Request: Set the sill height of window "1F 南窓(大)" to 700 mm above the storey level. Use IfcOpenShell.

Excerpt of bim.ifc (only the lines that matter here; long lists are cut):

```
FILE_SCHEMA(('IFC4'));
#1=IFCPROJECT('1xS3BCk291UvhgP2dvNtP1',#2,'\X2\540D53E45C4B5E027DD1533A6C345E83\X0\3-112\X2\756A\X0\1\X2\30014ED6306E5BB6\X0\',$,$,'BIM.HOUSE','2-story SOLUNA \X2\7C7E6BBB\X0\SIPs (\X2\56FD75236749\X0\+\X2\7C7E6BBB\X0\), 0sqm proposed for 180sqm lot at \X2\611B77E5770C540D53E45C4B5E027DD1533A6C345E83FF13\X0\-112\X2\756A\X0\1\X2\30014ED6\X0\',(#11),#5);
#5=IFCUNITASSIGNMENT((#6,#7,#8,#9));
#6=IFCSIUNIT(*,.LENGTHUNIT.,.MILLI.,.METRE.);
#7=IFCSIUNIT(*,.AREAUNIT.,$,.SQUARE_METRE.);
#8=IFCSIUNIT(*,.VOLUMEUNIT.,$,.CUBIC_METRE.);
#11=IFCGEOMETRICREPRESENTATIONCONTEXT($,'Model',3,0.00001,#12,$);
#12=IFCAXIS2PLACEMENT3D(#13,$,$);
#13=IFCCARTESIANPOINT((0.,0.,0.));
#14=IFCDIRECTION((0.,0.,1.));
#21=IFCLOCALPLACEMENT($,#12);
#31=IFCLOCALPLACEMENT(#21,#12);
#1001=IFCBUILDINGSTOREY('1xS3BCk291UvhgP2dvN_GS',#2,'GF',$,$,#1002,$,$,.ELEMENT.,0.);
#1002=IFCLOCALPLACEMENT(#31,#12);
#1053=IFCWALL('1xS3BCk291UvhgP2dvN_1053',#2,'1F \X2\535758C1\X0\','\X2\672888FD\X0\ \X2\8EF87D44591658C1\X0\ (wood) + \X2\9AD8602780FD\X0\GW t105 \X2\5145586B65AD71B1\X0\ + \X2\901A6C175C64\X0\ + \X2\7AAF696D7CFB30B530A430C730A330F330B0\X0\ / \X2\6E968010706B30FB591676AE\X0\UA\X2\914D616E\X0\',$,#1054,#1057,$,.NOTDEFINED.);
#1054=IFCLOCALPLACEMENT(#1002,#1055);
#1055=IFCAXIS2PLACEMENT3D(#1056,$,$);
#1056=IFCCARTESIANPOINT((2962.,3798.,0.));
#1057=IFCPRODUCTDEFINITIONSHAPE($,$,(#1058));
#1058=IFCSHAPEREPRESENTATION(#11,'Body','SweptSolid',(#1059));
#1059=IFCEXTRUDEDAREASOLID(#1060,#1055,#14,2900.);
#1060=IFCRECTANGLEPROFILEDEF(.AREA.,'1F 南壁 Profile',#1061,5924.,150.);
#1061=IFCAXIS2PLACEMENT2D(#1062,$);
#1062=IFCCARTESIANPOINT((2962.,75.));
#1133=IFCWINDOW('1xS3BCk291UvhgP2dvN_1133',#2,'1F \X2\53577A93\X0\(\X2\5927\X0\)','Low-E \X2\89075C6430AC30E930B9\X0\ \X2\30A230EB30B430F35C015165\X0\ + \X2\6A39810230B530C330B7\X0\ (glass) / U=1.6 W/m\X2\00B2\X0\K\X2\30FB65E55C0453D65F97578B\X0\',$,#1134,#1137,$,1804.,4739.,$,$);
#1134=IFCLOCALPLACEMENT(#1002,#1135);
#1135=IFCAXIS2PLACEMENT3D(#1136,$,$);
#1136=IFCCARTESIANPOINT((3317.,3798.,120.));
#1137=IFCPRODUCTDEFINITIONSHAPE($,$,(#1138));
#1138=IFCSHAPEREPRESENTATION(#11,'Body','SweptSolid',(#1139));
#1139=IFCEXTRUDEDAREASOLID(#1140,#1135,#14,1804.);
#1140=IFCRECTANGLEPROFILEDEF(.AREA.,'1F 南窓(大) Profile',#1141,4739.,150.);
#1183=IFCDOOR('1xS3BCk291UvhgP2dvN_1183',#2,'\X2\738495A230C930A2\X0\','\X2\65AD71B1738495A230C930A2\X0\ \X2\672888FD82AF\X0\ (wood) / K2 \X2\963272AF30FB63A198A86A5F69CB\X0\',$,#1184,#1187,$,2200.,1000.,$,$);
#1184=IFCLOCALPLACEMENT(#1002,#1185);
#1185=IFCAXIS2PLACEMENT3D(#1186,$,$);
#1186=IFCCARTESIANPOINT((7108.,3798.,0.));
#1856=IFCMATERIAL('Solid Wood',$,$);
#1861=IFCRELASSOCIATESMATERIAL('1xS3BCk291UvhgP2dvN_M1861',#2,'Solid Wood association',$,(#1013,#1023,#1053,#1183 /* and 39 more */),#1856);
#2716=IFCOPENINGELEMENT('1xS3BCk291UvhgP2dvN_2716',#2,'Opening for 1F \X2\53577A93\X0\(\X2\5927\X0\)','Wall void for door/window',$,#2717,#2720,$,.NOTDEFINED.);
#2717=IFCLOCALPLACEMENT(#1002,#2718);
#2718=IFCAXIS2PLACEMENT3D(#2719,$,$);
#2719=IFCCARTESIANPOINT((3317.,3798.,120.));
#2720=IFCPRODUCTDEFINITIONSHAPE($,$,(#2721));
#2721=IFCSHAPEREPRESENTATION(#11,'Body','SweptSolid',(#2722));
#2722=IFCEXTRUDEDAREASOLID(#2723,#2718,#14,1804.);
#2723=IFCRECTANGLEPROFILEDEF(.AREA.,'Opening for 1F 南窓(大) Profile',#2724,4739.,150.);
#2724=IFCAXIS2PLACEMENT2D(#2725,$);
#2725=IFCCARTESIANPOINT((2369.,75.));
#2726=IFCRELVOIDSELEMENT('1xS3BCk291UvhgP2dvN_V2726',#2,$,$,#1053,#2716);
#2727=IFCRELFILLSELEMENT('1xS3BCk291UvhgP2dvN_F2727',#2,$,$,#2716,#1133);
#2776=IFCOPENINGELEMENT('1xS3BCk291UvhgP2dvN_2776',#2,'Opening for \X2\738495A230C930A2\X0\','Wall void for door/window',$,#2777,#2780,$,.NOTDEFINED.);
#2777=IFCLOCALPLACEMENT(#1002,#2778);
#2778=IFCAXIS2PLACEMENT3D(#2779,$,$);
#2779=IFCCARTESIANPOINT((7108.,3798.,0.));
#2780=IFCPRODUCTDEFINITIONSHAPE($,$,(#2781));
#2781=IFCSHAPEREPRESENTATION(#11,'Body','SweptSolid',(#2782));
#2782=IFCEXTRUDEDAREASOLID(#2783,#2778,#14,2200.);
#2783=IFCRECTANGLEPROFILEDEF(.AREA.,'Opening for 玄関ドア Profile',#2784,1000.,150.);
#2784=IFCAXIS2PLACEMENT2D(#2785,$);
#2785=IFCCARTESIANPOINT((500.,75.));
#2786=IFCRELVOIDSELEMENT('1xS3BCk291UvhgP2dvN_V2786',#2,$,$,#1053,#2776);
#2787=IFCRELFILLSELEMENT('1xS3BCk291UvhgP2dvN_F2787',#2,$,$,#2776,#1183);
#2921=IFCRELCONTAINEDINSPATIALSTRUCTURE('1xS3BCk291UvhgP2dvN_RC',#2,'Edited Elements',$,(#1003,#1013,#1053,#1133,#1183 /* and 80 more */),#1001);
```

```python
import numpy as np
import ifcopenshell
import ifcopenshell.api.geometry
import ifcopenshell.geom
import ifcopenshell.util.element
import ifcopenshell.util.placement
import ifcopenshell.util.shape
import ifcopenshell.util.unit

model = ifcopenshell.open("bim.ifc")
unit_scale = ifcopenshell.util.unit.calculate_unit_scale(model)

window = model.by_guid("1xS3BCk291UvhgP2dvN_1133")
opening = window.FillsVoids[0].RelatingOpeningElement
storey = ifcopenshell.util.element.get_container(window, ifc_class="IfcBuildingStorey")
level = ifcopenshell.util.placement.get_local_placement(storey.ObjectPlacement)[2, 3]

# The opening's origin need not be at the sill, so measure its lowest point.
shape = ifcopenshell.geom.create_shape(ifcopenshell.geom.settings(), opening)
bottom = ifcopenshell.util.shape.get_shape_bottom_elevation(shape, shape.geometry) / unit_scale
dz = level + 0.7 / unit_scale - bottom

shift = np.array([0.0, 0.0, dz])
# The window is not placed relative to its opening, so move both.
for product in (opening, window):
    matrix = ifcopenshell.util.placement.get_local_placement(product.ObjectPlacement)
    matrix[:3, 3] += shift
    ifcopenshell.api.geometry.edit_object_placement(model, product=product, matrix=matrix, is_si=False)

print(f"moved by {dz * unit_scale:+.3f} m")

model.write("bim_rev.ifc")
```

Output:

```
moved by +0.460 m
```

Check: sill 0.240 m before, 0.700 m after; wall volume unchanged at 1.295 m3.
